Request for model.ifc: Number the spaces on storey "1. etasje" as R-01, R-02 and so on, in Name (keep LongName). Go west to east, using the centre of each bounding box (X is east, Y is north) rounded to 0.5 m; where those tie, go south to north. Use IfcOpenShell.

First a look at what the model holds.

```python
import ifcopenshell
import ifcopenshell.util.element
import ifcopenshell.util.placement

model = ifcopenshell.open("model.ifc")
print(model.schema)
storey = next(s for s in model.by_type("IfcBuildingStorey") if s.Name == "1. etasje")
spaces = [e for e in ifcopenshell.util.element.get_decomposition(storey) if e.is_a("IfcSpace")]
for e in sorted(spaces, key=lambda e: e.id()):
    origin = ifcopenshell.util.placement.get_local_placement(e.ObjectPlacement)[:3, 3]
    print(e.id(), e.Name, e.LongName, origin.round(2) + 0.0, sep=" | ")
```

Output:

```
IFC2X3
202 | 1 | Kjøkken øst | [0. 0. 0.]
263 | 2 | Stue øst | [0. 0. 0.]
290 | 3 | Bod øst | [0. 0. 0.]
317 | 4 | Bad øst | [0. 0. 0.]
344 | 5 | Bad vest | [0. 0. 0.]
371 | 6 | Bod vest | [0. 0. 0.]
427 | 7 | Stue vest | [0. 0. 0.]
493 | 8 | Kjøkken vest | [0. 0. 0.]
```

```python
import ifcopenshell
import ifcopenshell.geom
import ifcopenshell.util.element
import ifcopenshell.util.shape

model = ifcopenshell.open("model.ifc")
settings = ifcopenshell.geom.settings()
settings.set("use-world-coords", True)


def centre(element):
    shape = ifcopenshell.geom.create_shape(settings, element)
    return ifcopenshell.util.shape.get_bbox_centroid(shape.geometry)


storey = next(s for s in model.by_type("IfcBuildingStorey") if s.Name == "1. etasje")
spaces = [e for e in ifcopenshell.util.element.get_decomposition(storey) if e.is_a("IfcSpace")]

# Insertion points can sit at a corner or the storey origin, so sort by the geometry (in metres).
centres = {e: centre(e) for e in spaces}
spaces.sort(key=lambda e: (round(centres[e][0] / 0.5), centres[e][1]))

for i, e in enumerate(spaces, start=1):
    number = f"R-{i:02d}"
    e.Name = number
    print(e.id(), number)

model.write("model-out.ifc")
```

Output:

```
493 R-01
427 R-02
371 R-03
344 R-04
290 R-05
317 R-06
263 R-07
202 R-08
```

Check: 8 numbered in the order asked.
